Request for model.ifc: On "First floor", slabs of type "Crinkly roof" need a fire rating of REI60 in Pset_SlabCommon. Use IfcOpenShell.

First a look at what the model holds.

```python
import ifcopenshell
import ifcopenshell.util.element

model = ifcopenshell.open("model.ifc")
print(model.schema)
storey = next(s for s in model.by_type("IfcBuildingStorey") if s.Name == "First floor")
slabs = [e for e in ifcopenshell.util.element.get_decomposition(storey) if e.is_a("IfcSlab")]
seen = {}
for e in slabs:
    element_type = ifcopenshell.util.element.get_type(e)
    key = (element_type.Name if element_type != e and element_type else None, ifcopenshell.util.element.get_pset(e, "Pset_SlabCommon", "FireRating"))
    seen[key] = seen.get(key, 0) + 1
for (name, value), count in sorted(seen.items(), key=str):
    print(count, "x", name, "|", value)
```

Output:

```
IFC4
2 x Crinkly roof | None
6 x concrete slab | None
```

```python
import ifcopenshell
import ifcopenshell.api.pset
import ifcopenshell.util.element

model = ifcopenshell.open("model.ifc")

storey = next(s for s in model.by_type("IfcBuildingStorey") if s.Name == "First floor")
slabs = [e for e in ifcopenshell.util.element.get_decomposition(storey) if e.is_a("IfcSlab")]

count = 0
for e in slabs:
    element_type = ifcopenshell.util.element.get_type(e)
    if element_type in (None, e) or element_type.Name != "Crinkly roof":
        continue
    # add_pset returns the element's existing set when there is one.
    pset = ifcopenshell.api.pset.add_pset(model, product=e, name="Pset_SlabCommon")
    ifcopenshell.api.pset.edit_pset(model, pset=pset, properties={"FireRating": "REI60"})
    count += 1

print(count, "slabs updated")

model.write("model-out.ifc")
```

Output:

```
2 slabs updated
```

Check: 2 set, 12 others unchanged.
